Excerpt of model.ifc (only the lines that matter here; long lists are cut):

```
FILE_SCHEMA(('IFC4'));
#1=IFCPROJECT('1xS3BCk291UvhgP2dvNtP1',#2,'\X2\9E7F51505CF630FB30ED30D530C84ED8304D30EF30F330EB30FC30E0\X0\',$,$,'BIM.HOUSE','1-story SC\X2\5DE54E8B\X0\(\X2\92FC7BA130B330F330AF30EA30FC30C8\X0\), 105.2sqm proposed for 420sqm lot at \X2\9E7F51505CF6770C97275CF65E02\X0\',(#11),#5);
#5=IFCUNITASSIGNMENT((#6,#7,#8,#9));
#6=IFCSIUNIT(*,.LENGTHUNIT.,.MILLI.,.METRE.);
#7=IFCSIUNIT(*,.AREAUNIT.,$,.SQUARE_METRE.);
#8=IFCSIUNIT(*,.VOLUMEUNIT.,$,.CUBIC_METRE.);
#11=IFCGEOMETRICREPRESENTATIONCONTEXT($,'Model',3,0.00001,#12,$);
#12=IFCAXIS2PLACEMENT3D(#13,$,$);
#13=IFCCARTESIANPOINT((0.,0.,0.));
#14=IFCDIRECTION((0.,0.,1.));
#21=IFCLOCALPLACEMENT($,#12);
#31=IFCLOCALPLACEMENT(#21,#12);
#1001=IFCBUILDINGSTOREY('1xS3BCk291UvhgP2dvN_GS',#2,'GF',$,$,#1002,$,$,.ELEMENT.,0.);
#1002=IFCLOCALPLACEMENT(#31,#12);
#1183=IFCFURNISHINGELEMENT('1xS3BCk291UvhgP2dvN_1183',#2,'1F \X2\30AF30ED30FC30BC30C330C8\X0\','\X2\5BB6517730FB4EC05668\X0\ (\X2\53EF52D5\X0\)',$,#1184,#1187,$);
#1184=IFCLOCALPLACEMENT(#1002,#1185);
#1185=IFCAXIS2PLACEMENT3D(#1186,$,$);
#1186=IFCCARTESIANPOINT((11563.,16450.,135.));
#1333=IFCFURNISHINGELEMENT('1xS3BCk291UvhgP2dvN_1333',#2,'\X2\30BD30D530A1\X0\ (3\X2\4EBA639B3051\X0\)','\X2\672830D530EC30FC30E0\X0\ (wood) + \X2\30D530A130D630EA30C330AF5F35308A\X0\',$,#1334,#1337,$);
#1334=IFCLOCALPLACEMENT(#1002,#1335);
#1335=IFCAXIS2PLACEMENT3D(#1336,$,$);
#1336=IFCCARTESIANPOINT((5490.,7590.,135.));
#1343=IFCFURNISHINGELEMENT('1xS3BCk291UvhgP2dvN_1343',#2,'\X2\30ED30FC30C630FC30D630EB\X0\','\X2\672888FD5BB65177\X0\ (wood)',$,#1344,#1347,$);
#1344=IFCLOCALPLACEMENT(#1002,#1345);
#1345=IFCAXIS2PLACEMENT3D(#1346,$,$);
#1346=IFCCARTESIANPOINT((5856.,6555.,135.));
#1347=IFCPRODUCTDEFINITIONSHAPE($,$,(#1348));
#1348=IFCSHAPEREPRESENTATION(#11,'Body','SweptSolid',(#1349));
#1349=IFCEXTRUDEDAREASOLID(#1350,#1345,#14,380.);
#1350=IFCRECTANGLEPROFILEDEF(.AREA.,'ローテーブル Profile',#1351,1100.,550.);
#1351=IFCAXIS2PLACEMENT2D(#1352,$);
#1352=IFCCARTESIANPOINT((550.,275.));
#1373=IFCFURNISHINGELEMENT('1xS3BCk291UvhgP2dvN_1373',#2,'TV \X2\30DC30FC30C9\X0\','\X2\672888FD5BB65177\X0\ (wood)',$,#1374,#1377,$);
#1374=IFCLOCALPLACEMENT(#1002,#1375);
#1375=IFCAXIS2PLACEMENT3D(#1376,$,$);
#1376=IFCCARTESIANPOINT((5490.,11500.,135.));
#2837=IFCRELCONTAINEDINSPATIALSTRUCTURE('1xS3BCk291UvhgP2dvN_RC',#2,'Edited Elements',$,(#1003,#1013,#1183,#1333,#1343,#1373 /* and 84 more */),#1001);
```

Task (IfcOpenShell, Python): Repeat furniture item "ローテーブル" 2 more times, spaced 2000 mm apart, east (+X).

```python
import numpy as np
import ifcopenshell
import ifcopenshell.api.geometry
import ifcopenshell.api.root
import ifcopenshell.util.element
import ifcopenshell.util.placement
import ifcopenshell.util.unit

model = ifcopenshell.open("model.ifc")
unit_scale = ifcopenshell.util.unit.calculate_unit_scale(model)


def reuse_history(source, copy):
    """copy_class also copies each property set's owner history, people and application; keep the originals."""
    for rel in copy.IsDefinedBy:
        if rel.is_a("IfcRelDefinesByProperties") and (history := rel.RelatingPropertyDefinition.OwnerHistory):
            rel.RelatingPropertyDefinition.OwnerHistory = source.OwnerHistory
            ifcopenshell.util.element.remove_deep2(model, history)


source = model.by_guid("1xS3BCk291UvhgP2dvN_1343")
base = ifcopenshell.util.placement.get_local_placement(source.ObjectPlacement)
step = np.array([1.0, 0.0, 0.0]) * 2 / unit_scale

for i in range(1, 3):
    copy = ifcopenshell.api.root.copy_class(model, product=source)
    copy.Representation = ifcopenshell.util.element.copy_deep(
        model, source.Representation, exclude=["IfcGeometricRepresentationContext", "IfcRepresentationMap"]
    )
    reuse_history(source, copy)
    matrix = base.copy()
    matrix[:3, 3] += i * step
    print("added at", matrix[:3, 3].round(3) + 0.0)
    ifcopenshell.api.geometry.edit_object_placement(model, product=copy, matrix=matrix, is_si=False)

model.write("model_edited.ifc")
```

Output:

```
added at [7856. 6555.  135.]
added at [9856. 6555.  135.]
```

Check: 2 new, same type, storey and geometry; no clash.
